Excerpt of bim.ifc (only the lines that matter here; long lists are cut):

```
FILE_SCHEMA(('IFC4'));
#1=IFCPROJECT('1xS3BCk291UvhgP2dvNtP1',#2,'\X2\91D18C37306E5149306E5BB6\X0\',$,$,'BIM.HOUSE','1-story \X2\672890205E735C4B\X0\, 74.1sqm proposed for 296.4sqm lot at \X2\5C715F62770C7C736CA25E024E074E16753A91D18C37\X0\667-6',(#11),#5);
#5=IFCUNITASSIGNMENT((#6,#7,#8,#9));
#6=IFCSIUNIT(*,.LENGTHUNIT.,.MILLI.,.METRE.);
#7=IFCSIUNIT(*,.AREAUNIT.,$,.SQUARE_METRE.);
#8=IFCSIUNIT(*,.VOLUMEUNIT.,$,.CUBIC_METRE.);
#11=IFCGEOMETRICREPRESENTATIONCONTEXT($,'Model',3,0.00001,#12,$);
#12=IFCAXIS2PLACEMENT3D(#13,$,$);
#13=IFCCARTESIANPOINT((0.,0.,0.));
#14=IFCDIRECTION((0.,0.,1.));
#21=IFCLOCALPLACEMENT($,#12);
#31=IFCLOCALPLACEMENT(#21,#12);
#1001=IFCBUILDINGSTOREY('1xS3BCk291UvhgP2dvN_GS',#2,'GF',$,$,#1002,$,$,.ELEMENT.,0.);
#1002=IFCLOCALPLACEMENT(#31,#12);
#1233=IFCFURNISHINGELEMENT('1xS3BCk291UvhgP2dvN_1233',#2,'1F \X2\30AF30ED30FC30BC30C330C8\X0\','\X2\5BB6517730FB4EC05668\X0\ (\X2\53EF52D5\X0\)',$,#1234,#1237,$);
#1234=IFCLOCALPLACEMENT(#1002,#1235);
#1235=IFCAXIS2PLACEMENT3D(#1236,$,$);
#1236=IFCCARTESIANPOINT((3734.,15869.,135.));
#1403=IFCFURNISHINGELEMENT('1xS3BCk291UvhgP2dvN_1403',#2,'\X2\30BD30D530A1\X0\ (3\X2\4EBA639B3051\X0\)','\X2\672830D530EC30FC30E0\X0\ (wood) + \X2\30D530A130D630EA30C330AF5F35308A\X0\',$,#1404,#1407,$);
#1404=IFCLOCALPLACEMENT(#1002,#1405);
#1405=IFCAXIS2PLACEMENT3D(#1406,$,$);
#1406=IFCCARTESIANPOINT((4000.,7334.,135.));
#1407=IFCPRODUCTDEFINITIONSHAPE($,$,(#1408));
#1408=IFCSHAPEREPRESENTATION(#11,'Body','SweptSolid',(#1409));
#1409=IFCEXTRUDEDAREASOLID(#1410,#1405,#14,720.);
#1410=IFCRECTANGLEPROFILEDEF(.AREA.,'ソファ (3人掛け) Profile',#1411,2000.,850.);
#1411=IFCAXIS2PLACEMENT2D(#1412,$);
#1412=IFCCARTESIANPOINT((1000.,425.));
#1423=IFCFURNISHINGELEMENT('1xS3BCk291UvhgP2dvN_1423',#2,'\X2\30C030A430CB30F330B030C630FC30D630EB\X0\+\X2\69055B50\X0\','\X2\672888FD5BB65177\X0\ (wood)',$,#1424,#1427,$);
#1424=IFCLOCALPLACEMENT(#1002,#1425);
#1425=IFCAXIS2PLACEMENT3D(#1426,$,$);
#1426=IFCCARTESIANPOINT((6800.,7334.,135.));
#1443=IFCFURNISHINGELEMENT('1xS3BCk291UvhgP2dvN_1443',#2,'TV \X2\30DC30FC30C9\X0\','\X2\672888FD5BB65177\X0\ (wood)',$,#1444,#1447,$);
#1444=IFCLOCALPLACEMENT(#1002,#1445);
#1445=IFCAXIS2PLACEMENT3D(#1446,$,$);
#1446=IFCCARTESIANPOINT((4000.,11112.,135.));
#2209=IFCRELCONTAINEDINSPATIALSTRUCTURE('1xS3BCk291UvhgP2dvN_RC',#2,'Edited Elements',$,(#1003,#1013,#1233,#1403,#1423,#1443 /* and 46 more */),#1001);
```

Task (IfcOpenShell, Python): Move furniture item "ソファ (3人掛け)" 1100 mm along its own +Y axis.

```python
import ifcopenshell
import ifcopenshell.api.geometry
import ifcopenshell.util.placement
import ifcopenshell.util.unit

model = ifcopenshell.open("bim.ifc")
unit_scale = ifcopenshell.util.unit.calculate_unit_scale(model)

item = model.by_id(1403)
matrix = ifcopenshell.util.placement.get_local_placement(item.ObjectPlacement)
matrix[:3, 3] += matrix[:3, 1] * 1.1 / unit_scale
ifcopenshell.api.geometry.edit_object_placement(model, product=item, matrix=matrix, is_si=False)

print(ifcopenshell.util.placement.get_local_placement(item.ObjectPlacement).round(3) + 0.0)

model.write("bim_v2.ifc")
```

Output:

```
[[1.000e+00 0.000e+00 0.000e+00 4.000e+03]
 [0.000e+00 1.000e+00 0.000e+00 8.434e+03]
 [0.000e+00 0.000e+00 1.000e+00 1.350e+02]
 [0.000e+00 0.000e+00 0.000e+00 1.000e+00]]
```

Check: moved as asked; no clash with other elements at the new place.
